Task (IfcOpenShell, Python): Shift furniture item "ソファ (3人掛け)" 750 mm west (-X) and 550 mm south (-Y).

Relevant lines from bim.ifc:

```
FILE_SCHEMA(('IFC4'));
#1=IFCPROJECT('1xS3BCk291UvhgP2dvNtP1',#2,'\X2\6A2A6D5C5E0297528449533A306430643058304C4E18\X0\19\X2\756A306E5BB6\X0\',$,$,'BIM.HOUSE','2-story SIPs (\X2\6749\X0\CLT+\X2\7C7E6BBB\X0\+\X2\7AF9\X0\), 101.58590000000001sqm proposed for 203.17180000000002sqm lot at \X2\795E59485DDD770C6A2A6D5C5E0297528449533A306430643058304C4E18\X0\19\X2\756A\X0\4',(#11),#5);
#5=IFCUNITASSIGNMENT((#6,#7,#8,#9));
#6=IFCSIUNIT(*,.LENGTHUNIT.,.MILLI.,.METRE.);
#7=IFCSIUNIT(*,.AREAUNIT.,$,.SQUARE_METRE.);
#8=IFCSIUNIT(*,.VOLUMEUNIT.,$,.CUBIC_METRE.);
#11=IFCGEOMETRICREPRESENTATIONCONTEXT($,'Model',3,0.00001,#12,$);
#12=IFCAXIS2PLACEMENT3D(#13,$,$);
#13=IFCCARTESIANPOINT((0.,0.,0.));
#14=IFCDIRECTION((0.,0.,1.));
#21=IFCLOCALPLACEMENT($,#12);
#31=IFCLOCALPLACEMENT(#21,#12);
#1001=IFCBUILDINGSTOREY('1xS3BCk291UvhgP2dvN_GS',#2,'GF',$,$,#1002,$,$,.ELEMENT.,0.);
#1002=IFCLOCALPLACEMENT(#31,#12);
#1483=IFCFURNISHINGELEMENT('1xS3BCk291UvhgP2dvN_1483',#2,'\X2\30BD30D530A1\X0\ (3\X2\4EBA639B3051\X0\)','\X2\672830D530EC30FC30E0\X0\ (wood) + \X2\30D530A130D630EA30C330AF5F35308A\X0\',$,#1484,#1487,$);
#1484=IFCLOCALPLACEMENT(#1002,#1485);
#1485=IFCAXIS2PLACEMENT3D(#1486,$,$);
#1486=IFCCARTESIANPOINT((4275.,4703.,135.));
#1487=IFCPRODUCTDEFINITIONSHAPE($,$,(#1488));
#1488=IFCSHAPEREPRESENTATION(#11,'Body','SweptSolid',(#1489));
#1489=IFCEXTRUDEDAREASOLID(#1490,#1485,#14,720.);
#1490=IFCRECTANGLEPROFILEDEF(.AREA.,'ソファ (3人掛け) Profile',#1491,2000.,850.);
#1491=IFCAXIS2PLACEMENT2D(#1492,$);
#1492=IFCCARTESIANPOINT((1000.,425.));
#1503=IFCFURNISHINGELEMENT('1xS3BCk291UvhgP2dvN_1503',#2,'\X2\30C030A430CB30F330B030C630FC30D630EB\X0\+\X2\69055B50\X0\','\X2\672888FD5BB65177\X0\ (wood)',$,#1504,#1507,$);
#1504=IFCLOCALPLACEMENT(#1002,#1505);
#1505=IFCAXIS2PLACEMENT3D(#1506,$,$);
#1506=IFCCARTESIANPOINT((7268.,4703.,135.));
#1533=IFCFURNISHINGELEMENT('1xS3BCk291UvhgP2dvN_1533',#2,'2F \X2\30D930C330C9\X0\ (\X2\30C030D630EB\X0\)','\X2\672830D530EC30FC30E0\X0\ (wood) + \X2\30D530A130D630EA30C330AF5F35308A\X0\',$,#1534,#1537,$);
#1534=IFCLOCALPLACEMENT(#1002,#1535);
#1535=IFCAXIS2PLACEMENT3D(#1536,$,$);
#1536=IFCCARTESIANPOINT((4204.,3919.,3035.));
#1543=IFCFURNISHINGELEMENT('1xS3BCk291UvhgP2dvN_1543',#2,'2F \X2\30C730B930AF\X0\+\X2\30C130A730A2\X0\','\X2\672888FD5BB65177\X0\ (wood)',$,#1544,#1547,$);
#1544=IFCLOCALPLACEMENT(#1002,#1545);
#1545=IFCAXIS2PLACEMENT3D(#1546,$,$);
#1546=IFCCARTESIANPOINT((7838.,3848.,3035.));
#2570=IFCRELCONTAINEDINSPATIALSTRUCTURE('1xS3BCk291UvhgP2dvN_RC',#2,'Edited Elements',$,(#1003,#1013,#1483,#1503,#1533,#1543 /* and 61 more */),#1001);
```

```python
import ifcopenshell
import ifcopenshell.api.geometry
import ifcopenshell.util.placement

model = ifcopenshell.open("bim.ifc")

item = model.by_guid("1xS3BCk291UvhgP2dvN_1483")
matrix = ifcopenshell.util.placement.get_local_placement(item.ObjectPlacement)
matrix[0, 3] -= 750.0
matrix[1, 3] -= 550.0
ifcopenshell.api.geometry.edit_object_placement(model, product=item, matrix=matrix, is_si=False)

print(ifcopenshell.util.placement.get_local_placement(item.ObjectPlacement).round(3) + 0.0)

model.write("bim_rev.ifc")
```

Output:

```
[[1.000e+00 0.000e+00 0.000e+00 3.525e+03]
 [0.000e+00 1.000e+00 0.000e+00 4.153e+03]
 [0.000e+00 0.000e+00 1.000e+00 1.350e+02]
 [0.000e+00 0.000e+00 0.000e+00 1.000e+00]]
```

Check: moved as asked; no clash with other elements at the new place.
